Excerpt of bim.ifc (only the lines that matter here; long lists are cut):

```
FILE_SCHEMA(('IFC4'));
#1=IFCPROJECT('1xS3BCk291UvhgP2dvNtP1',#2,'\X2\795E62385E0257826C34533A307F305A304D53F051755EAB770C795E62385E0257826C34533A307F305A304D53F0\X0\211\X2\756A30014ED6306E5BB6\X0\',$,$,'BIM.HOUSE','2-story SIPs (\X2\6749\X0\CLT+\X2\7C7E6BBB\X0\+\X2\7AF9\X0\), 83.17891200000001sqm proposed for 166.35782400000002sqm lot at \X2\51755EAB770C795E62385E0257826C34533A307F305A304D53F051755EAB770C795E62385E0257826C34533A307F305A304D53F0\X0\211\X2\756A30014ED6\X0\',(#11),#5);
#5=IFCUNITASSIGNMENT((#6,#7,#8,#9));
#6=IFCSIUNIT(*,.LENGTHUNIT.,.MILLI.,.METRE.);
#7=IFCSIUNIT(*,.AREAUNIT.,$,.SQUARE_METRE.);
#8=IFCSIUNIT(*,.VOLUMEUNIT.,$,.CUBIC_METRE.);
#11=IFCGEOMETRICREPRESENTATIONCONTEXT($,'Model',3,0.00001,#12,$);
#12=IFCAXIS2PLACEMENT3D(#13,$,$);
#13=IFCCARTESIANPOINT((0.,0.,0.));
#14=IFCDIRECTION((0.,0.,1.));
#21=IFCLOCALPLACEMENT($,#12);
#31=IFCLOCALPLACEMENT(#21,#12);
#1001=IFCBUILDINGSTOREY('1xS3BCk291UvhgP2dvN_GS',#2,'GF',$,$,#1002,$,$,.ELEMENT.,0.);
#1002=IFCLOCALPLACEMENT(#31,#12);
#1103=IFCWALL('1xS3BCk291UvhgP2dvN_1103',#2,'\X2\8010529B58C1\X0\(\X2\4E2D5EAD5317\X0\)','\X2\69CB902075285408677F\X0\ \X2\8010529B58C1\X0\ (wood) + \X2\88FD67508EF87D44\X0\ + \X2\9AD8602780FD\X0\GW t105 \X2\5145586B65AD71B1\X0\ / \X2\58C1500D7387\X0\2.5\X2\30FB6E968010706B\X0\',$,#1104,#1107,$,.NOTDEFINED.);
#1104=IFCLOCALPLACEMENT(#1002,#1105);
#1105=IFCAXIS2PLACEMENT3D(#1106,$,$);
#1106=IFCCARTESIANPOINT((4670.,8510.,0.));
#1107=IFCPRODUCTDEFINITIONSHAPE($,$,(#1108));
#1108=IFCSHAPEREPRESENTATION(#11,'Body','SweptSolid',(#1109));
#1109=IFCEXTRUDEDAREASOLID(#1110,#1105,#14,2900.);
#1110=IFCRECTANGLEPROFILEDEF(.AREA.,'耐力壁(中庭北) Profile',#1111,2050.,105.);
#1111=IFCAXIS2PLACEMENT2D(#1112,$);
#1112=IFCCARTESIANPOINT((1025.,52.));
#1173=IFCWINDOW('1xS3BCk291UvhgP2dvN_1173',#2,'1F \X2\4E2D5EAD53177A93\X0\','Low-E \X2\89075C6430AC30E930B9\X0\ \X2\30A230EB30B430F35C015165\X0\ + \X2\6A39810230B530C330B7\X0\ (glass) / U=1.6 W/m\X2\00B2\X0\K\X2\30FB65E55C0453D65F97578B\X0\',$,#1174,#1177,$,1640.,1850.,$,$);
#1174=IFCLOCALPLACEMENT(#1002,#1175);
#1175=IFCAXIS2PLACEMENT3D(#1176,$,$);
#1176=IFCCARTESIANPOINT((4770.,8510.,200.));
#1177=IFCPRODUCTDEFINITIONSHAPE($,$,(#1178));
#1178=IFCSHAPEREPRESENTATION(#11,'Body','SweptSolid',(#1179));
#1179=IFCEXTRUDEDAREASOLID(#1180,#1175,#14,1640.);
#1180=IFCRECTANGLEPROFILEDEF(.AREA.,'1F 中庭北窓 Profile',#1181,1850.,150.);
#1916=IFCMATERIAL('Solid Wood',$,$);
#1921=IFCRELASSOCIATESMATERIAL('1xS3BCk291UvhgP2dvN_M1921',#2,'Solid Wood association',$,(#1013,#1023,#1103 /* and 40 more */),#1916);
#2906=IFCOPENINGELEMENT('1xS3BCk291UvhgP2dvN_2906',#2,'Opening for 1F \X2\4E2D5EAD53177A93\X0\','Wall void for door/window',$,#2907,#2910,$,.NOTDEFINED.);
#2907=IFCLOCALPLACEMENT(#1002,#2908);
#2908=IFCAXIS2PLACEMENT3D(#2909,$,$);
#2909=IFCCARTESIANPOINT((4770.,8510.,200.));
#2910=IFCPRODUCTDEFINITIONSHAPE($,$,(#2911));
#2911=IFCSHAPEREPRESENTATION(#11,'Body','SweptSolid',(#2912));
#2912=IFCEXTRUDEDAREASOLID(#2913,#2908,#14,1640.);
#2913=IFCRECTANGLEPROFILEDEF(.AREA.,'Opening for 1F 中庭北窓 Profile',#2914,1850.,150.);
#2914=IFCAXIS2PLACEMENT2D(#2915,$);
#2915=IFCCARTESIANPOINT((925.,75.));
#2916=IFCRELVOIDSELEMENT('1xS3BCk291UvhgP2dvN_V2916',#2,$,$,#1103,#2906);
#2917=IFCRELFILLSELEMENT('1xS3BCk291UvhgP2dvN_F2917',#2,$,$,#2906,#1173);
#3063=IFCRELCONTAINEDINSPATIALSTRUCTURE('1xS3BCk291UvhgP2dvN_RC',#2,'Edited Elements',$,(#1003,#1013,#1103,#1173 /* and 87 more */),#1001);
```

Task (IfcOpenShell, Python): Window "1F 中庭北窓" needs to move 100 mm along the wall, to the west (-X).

```python
import ifcopenshell
import ifcopenshell.api.geometry
import ifcopenshell.util.placement

model = ifcopenshell.open("bim.ifc")

window = model.by_guid("1xS3BCk291UvhgP2dvN_1173")
opening = window.FillsVoids[0].RelatingOpeningElement
wall = opening.VoidsElements[0].RelatingBuildingElement

wall_matrix = ifcopenshell.util.placement.get_local_placement(wall.ObjectPlacement)
shift = wall_matrix[:3, 0] * -100.0
before = ifcopenshell.util.placement.get_local_placement(window.ObjectPlacement)[:3, 3].copy()

# The window is not placed relative to its opening, so move both.
for product in (opening, window):
    matrix = ifcopenshell.util.placement.get_local_placement(product.ObjectPlacement)
    matrix[:3, 3] += shift
    ifcopenshell.api.geometry.edit_object_placement(model, product=product, matrix=matrix, is_si=False)

after = ifcopenshell.util.placement.get_local_placement(window.ObjectPlacement)[:3, 3]
print("window moved by", (after - before).round(3) + 0.0)

model.write("bim_v2.ifc")
```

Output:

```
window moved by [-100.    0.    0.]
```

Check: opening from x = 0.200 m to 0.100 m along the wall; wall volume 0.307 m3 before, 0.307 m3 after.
